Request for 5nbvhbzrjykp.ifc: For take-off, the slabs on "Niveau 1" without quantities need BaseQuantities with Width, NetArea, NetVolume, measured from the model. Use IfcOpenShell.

First a look at what the model holds.

```python
import ifcopenshell
import ifcopenshell.util.element
import ifcopenshell.util.unit

model = ifcopenshell.open("5nbvhbzrjykp.ifc")
print(model.schema)
for unit_type in ("LENGTHUNIT", "AREAUNIT", "VOLUMEUNIT"):
    print(unit_type, ifcopenshell.util.unit.calculate_unit_scale(model, unit_type))
storey = next(s for s in model.by_type("IfcBuildingStorey") if s.Name == "Niveau 1")
slabs = [e for e in ifcopenshell.util.element.get_decomposition(storey) if e.is_a("IfcSlab")]
for e in sorted(slabs, key=lambda e: e.id()):
    print(e.id(), e.is_a(), e.Name, list(ifcopenshell.util.element.get_psets(e, qtos_only=True)), sep=" | ")
```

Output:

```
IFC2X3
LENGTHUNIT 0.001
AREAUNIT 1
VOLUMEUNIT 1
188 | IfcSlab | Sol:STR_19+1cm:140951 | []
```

```python
import ifcopenshell
import ifcopenshell.api.pset
import ifcopenshell.geom
import ifcopenshell.util.element
import ifcopenshell.util.shape
import ifcopenshell.util.unit

model = ifcopenshell.open("5nbvhbzrjykp.ifc")
unit_scale = ifcopenshell.util.unit.calculate_unit_scale(model)
area_scale = ifcopenshell.util.unit.calculate_unit_scale(model, "AREAUNIT")
volume_scale = ifcopenshell.util.unit.calculate_unit_scale(model, "VOLUMEUNIT")
settings = ifcopenshell.geom.settings()

storey = next(s for s in model.by_type("IfcBuildingStorey") if s.Name == "Niveau 1")
slabs = [e for e in ifcopenshell.util.element.get_decomposition(storey) if e.is_a("IfcSlab")]

for e in sorted(slabs, key=lambda e: e.id()):
    if ifcopenshell.util.element.get_psets(e, qtos_only=True, should_inherit=False):
        continue
    # Geometry comes back in metres, in the element's own axes.
    shape = ifcopenshell.geom.create_shape(settings, e)
    values = {
        "Width": ifcopenshell.util.shape.get_z(shape.geometry) / unit_scale,
        "NetArea": ifcopenshell.util.shape.get_footprint_area(shape.geometry) / area_scale,
        "NetVolume": ifcopenshell.util.shape.get_volume(shape.geometry) / volume_scale,
    }
    qto = ifcopenshell.api.pset.add_qto(model, product=e, name="BaseQuantities")
    ifcopenshell.api.pset.edit_qto(model, qto=qto, properties=values)
    print(e.id(), {k: round(v, 3) for k, v in values.items()})

model.write("5nbvhbzrjykp_rev.ifc")
```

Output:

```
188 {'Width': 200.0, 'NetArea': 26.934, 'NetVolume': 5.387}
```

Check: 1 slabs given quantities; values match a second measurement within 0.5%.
